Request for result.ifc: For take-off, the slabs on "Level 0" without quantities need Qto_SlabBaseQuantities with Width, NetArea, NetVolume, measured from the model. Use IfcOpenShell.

First a look at what the model holds.

```python
import ifcopenshell
import ifcopenshell.util.element
import ifcopenshell.util.unit

model = ifcopenshell.open("result.ifc")
print(model.schema)
for unit_type in ("LENGTHUNIT", "AREAUNIT", "VOLUMEUNIT"):
    print(unit_type, ifcopenshell.util.unit.calculate_unit_scale(model, unit_type))
storey = next(s for s in model.by_type("IfcBuildingStorey") if s.Name == "Level 0")
slabs = [e for e in ifcopenshell.util.element.get_decomposition(storey) if e.is_a("IfcSlab")]
for e in sorted(slabs, key=lambda e: e.id()):
    print(e.id(), e.is_a(), e.Name, list(ifcopenshell.util.element.get_psets(e, qtos_only=True)), sep=" | ")
```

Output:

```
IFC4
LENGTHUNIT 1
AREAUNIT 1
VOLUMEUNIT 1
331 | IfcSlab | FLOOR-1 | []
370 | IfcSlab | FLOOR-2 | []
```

```python
import ifcopenshell
import ifcopenshell.api.pset
import ifcopenshell.geom
import ifcopenshell.util.element
import ifcopenshell.util.shape
import ifcopenshell.util.unit

model = ifcopenshell.open("result.ifc")
unit_scale = ifcopenshell.util.unit.calculate_unit_scale(model)
area_scale = ifcopenshell.util.unit.calculate_unit_scale(model, "AREAUNIT")
volume_scale = ifcopenshell.util.unit.calculate_unit_scale(model, "VOLUMEUNIT")
settings = ifcopenshell.geom.settings()

storey = next(s for s in model.by_type("IfcBuildingStorey") if s.Name == "Level 0")
slabs = [e for e in ifcopenshell.util.element.get_decomposition(storey) if e.is_a("IfcSlab")]

for e in sorted(slabs, key=lambda e: e.id()):
    if ifcopenshell.util.element.get_psets(e, qtos_only=True, should_inherit=False):
        continue
    # Geometry comes back in metres, in the element's own axes.
    shape = ifcopenshell.geom.create_shape(settings, e)
    values = {
        "Width": ifcopenshell.util.shape.get_z(shape.geometry) / unit_scale,
        "NetArea": ifcopenshell.util.shape.get_footprint_area(shape.geometry) / area_scale,
        "NetVolume": ifcopenshell.util.shape.get_volume(shape.geometry) / volume_scale,
    }
    qto = ifcopenshell.api.pset.add_qto(model, product=e, name="Qto_SlabBaseQuantities")
    ifcopenshell.api.pset.edit_qto(model, qto=qto, properties=values)
    print(e.id(), {k: round(v, 3) for k, v in values.items()})

model.write("result_edited.ifc")
```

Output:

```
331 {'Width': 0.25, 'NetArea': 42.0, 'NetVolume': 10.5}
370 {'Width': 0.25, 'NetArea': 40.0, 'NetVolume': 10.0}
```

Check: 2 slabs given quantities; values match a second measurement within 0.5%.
